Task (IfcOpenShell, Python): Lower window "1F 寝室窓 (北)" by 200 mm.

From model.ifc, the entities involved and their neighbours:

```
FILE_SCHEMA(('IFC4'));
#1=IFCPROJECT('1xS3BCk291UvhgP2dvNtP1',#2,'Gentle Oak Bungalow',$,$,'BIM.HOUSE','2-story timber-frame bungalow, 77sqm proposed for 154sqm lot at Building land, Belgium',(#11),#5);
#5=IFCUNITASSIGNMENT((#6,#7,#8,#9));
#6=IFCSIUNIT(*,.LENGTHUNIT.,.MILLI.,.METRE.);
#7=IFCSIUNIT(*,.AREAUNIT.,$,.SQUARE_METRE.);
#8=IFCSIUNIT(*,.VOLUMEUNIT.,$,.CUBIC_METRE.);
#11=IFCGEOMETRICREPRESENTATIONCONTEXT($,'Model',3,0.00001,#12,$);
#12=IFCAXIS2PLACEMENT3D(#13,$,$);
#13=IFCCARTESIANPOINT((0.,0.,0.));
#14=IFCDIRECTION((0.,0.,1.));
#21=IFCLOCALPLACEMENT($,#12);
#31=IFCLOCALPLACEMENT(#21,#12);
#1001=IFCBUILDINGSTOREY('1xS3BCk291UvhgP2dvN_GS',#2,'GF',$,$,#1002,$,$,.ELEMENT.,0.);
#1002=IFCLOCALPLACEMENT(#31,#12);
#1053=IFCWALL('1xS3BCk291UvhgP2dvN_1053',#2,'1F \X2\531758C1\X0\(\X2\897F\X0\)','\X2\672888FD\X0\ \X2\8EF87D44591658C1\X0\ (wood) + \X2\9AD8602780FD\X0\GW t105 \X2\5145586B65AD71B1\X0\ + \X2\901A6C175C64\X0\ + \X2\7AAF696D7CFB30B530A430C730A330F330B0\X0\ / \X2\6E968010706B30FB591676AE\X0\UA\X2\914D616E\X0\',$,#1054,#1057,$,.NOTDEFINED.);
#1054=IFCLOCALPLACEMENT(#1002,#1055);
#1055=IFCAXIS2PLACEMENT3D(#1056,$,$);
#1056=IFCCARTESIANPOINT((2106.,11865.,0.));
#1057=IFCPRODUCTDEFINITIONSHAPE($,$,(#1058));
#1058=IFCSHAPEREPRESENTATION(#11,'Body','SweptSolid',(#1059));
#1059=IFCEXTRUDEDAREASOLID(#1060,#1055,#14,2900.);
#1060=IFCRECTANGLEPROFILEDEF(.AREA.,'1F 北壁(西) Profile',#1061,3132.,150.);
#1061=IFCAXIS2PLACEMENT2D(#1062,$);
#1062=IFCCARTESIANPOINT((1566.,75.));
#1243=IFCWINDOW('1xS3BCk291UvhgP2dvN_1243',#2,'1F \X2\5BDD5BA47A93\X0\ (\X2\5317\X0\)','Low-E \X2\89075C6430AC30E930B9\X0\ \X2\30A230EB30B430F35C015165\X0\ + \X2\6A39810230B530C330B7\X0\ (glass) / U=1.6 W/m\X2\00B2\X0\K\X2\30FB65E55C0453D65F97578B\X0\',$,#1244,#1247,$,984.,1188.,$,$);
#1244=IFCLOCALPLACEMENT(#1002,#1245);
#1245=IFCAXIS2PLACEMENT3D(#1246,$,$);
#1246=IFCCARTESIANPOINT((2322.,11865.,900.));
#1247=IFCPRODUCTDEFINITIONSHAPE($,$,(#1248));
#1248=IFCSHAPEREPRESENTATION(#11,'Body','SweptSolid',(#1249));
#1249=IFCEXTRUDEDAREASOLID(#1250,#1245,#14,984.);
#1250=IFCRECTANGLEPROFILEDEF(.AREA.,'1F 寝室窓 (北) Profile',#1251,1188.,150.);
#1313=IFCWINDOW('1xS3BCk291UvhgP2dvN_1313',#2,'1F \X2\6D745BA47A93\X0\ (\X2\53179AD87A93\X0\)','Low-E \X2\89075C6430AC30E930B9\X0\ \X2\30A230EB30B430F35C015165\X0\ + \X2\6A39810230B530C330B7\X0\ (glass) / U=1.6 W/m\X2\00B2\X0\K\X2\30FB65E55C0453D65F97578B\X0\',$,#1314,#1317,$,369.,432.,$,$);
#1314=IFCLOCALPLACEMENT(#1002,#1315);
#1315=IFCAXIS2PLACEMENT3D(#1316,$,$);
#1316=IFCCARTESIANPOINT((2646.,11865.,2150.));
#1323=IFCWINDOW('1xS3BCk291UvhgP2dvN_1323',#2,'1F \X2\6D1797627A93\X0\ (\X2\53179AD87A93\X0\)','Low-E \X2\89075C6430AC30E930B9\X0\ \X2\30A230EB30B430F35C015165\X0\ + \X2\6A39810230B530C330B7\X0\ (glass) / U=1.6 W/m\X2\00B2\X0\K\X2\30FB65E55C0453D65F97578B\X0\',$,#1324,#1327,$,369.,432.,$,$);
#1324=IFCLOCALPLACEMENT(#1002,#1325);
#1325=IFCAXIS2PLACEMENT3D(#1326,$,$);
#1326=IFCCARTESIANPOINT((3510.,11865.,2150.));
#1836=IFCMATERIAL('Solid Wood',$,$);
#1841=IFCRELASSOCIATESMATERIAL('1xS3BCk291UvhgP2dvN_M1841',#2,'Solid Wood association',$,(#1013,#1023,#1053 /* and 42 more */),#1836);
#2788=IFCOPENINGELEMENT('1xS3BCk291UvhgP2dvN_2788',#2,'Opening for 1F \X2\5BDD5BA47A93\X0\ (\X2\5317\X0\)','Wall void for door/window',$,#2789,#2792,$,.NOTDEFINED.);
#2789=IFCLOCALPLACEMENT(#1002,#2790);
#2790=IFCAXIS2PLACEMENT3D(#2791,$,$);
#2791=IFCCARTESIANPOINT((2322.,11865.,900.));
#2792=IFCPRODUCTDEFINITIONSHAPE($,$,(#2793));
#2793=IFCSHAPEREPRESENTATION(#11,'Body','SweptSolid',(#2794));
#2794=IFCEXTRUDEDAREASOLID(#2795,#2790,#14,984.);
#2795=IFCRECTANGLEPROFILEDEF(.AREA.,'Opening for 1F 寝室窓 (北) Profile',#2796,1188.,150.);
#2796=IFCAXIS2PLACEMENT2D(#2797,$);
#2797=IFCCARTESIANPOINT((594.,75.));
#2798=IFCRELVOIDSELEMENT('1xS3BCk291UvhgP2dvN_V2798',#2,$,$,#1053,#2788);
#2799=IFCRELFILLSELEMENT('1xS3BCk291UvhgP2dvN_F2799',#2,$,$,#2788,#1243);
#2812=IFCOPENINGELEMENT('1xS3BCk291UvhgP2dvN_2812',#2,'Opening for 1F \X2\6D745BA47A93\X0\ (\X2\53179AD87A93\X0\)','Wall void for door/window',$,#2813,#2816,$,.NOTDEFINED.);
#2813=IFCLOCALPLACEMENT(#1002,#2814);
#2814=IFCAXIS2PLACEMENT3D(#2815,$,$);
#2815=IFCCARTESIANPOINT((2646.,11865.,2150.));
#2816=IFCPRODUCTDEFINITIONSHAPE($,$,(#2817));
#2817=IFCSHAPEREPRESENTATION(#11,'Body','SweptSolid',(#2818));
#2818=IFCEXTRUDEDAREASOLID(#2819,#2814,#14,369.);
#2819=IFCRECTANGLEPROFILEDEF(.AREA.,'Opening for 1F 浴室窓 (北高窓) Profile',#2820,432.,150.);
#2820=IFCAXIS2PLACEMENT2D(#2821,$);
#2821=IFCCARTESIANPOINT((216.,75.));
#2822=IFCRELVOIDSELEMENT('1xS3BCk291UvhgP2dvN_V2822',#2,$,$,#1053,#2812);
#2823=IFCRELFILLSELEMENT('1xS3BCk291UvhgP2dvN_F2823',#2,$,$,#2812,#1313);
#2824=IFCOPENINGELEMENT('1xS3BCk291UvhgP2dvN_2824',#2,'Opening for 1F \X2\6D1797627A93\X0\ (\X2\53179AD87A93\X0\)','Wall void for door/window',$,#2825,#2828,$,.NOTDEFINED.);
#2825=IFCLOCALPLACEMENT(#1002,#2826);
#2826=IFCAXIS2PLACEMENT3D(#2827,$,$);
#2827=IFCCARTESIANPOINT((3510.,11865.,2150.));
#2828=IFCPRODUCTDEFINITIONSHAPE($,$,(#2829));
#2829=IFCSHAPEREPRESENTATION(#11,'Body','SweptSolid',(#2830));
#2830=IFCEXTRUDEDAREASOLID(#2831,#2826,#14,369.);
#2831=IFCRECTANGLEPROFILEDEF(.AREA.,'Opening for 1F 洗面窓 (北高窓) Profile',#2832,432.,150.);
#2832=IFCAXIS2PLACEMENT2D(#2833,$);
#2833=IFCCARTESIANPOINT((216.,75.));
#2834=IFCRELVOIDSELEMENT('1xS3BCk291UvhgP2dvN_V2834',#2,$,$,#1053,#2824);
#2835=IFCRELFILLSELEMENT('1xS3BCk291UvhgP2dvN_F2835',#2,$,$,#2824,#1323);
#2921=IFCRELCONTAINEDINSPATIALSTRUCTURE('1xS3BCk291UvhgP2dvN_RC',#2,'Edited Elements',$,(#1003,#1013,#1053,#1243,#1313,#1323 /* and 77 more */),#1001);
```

```python
import numpy as np
import ifcopenshell
import ifcopenshell.api.geometry
import ifcopenshell.util.placement
import ifcopenshell.util.unit

model = ifcopenshell.open("model.ifc")
unit_scale = ifcopenshell.util.unit.calculate_unit_scale(model)

window = model.by_id(1243)
opening = window.FillsVoids[0].RelatingOpeningElement
dz = -0.2 / unit_scale

shift = np.array([0.0, 0.0, dz])
# The window is not placed relative to its opening, so move both.
for product in (opening, window):
    matrix = ifcopenshell.util.placement.get_local_placement(product.ObjectPlacement)
    matrix[:3, 3] += shift
    ifcopenshell.api.geometry.edit_object_placement(model, product=product, matrix=matrix, is_si=False)

print(f"moved by {dz * unit_scale:+.3f} m")

model.write("model_updated.ifc")
```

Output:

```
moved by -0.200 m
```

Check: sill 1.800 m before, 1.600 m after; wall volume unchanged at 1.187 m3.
